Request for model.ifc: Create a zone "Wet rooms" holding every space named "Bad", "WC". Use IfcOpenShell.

First a look at what the model holds.

```python
import ifcopenshell

model = ifcopenshell.open("model.ifc")
print(model.schema)
seen = {}
for space in model.by_type("IfcSpace"):
    seen[space.LongName] = seen.get(space.LongName, 0) + 1
for name, count in sorted(seen.items(), key=str):
    print(count, "x", name)
print("zones:", [z.Name for z in model.by_type("IfcZone")][:20])
```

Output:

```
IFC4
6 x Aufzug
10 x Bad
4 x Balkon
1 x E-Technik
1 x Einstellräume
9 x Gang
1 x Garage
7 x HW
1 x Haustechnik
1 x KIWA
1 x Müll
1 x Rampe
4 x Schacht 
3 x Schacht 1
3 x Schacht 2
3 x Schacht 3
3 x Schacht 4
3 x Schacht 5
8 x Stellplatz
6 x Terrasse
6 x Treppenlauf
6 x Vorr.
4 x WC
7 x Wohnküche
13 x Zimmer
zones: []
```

```python
import ifcopenshell
import ifcopenshell.api.group
import ifcopenshell.api.root

model = ifcopenshell.open("model.ifc")

names = {"Bad", "WC"}
spaces = [s for s in model.by_type("IfcSpace") if s.LongName in names]

zone = ifcopenshell.api.root.create_entity(model, ifc_class="IfcZone", name="Wet rooms")
ifcopenshell.api.group.assign_group(model, products=spaces, group=zone)
print(len(spaces), "spaces in", zone.Name)

model.write("model_updated.ifc")
```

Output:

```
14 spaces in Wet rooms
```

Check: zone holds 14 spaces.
